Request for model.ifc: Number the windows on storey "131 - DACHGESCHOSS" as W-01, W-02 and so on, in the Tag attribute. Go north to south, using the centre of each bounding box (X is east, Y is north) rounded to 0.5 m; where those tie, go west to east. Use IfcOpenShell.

First a look at what the model holds.

```python
import ifcopenshell
import ifcopenshell.util.element
import ifcopenshell.util.placement

model = ifcopenshell.open("model.ifc")
print(model.schema)
storey = next(s for s in model.by_type("IfcBuildingStorey") if s.Name == "131 - DACHGESCHOSS")
windows = [e for e in ifcopenshell.util.element.get_decomposition(storey) if e.is_a("IfcWindow")]
for e in sorted(windows, key=lambda e: e.id()):
    origin = ifcopenshell.util.placement.get_local_placement(e.ObjectPlacement)[:3, 3]
    print(e.id(), e.Tag, e.Name, origin.round(2) + 0.0, sep=" | ")
```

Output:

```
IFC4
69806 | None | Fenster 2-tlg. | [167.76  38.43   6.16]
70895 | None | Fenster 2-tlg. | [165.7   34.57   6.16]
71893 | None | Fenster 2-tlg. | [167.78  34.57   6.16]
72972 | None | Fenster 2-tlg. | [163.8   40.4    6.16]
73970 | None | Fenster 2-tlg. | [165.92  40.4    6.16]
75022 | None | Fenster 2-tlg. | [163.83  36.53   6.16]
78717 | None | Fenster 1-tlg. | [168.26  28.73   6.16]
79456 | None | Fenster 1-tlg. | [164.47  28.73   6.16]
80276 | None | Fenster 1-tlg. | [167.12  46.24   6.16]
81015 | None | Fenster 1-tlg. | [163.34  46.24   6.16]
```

```python
import ifcopenshell
import ifcopenshell.geom
import ifcopenshell.util.element
import ifcopenshell.util.shape

model = ifcopenshell.open("model.ifc")
settings = ifcopenshell.geom.settings()
settings.set("use-world-coords", True)


def centre(element):
    shape = ifcopenshell.geom.create_shape(settings, element)
    return ifcopenshell.util.shape.get_bbox_centroid(shape.geometry)


storey = next(s for s in model.by_type("IfcBuildingStorey") if s.Name == "131 - DACHGESCHOSS")
windows = [e for e in ifcopenshell.util.element.get_decomposition(storey) if e.is_a("IfcWindow")]

# Insertion points can sit at a corner or the storey origin, so sort by the geometry (in metres).
centres = {e: centre(e) for e in windows}
windows.sort(key=lambda e: (-round(centres[e][1] / 0.5), centres[e][0]))

for i, e in enumerate(windows, start=1):
    number = f"W-{i:02d}"
    e.Tag = number
    print(e.id(), number)

model.write("model_v2.ifc")
```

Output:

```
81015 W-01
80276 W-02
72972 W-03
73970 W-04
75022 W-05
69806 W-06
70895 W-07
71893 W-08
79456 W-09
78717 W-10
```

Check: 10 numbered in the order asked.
